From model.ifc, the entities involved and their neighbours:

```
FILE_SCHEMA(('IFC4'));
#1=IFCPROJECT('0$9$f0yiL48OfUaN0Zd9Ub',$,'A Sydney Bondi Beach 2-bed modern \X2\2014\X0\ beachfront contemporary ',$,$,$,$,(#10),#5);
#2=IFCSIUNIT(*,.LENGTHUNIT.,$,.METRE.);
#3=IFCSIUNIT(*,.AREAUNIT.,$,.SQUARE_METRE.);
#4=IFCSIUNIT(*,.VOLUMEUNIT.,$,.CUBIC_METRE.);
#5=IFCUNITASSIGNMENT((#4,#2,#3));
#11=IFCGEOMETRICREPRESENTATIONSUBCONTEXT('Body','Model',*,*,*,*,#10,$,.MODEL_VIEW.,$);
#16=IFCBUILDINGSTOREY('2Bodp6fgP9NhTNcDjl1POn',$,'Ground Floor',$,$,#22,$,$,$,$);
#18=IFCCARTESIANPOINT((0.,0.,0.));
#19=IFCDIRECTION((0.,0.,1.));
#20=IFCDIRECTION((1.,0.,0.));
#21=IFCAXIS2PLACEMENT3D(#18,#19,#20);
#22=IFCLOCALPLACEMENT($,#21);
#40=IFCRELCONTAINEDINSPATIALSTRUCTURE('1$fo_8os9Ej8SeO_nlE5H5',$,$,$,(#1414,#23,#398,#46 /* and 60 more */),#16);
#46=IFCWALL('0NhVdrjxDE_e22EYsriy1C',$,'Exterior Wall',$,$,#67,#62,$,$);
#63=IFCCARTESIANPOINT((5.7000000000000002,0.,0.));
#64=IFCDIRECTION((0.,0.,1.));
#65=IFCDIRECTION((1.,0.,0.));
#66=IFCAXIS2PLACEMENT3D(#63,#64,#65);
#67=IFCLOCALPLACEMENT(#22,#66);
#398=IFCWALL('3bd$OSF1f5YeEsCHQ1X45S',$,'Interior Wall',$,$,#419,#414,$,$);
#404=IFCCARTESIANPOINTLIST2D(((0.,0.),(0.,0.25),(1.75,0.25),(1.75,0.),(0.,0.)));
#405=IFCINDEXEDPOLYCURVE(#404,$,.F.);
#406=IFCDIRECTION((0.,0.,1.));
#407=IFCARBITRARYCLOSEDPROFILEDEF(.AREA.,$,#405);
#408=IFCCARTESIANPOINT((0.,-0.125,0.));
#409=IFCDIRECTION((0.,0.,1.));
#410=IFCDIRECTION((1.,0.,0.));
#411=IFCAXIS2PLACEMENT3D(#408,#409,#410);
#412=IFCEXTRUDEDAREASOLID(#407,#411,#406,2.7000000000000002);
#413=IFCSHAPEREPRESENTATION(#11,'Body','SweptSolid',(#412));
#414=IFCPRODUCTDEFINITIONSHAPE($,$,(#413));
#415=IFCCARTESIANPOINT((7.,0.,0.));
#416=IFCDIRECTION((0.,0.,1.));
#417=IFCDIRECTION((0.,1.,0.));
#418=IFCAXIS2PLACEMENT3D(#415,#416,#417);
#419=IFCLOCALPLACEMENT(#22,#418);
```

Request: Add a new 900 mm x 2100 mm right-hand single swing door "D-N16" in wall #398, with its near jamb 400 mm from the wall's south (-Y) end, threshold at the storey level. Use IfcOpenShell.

```python
import numpy as np
import ifcopenshell
import ifcopenshell.api.feature
import ifcopenshell.api.geometry
import ifcopenshell.api.root
import ifcopenshell.api.spatial
import ifcopenshell.geom
import ifcopenshell.util.element
import ifcopenshell.util.placement
import ifcopenshell.util.representation
import ifcopenshell.util.shape
import ifcopenshell.util.unit

model = ifcopenshell.open("model.ifc")
unit_scale = ifcopenshell.util.unit.calculate_unit_scale(model)
settings = ifcopenshell.geom.settings()


def volume(element):
    """Net volume in cubic metres, openings subtracted."""
    shape = ifcopenshell.geom.create_shape(settings, element)
    return ifcopenshell.util.shape.get_volume(shape.geometry)


wall = model.by_guid("3bd$OSF1f5YeEsCHQ1X45S")
storey = ifcopenshell.util.element.get_container(wall, ifc_class="IfcBuildingStorey")
context = ifcopenshell.util.representation.get_context(model, "Model", "Body", "MODEL_VIEW")
before = volume(wall)

width, height, from_end, sill = 0.9, 2.1, 0.4, 0.0  # metres

# The wall runs along its own X axis, and the end named is its -X end.
wall_shape = ifcopenshell.geom.create_shape(settings, wall)
x, y, z = ifcopenshell.util.shape.get_vertices(wall_shape.geometry).T
start = x.min() + from_end
face, thickness = float(y.min()), float(y.max() - y.min())
wall_matrix = ifcopenshell.util.placement.get_local_placement(wall.ObjectPlacement)
level = ifcopenshell.util.placement.get_local_placement(storey.ObjectPlacement)[2, 3]


def in_wall(x, y):
    """Placement at x, y metres in the wall's axes, at sill height."""
    matrix = wall_matrix.copy()
    matrix[:, 3] = wall_matrix @ np.array([x / unit_scale, y / unit_scale, 0.0, 1.0])
    matrix[2, 3] = level + sill / unit_scale
    return matrix


# Opening: a box that overshoots both wall faces by 50 mm.
opening = ifcopenshell.api.root.create_entity(model, ifc_class="IfcOpeningElement", predefined_type="OPENING")
box = ifcopenshell.api.geometry.add_wall_representation(
    model, context=context, length=width, height=height, thickness=thickness + 0.1
)
ifcopenshell.api.geometry.assign_representation(model, product=opening, representation=box)
ifcopenshell.api.geometry.edit_object_placement(model, product=opening, matrix=in_wall(start, face - 0.05), is_si=False)
ifcopenshell.api.feature.add_feature(model, feature=opening, element=wall)

door = ifcopenshell.api.root.create_entity(model, ifc_class="IfcDoor", name="D-N16", predefined_type="DOOR")
door.OverallWidth, door.OverallHeight = width / unit_scale, height / unit_scale
door.OperationType = "SINGLE_SWING_RIGHT"
body = ifcopenshell.api.geometry.add_door_representation(
    model,
    context=context,
    overall_width=door.OverallWidth,
    overall_height=door.OverallHeight,
    operation_type="SINGLE_SWING_RIGHT",
    lining_properties={"LiningDepth": thickness / unit_scale, "ThresholdDepth": thickness / unit_scale},
)
ifcopenshell.api.geometry.assign_representation(model, product=door, representation=body)
ifcopenshell.api.spatial.assign_container(model, products=[door], relating_structure=storey)
ifcopenshell.api.feature.add_filling(model, opening=opening, element=door)

# The lining spans the wall, so the door starts at the wall face.
ifcopenshell.api.geometry.edit_object_placement(model, product=door, matrix=in_wall(start, face), is_si=False)

after = volume(wall)

print(f"wall volume {before:.3f} -> {after:.3f} m3")

model.write("model_rev.ifc")
```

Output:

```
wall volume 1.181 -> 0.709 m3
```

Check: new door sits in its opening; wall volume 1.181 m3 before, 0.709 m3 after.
